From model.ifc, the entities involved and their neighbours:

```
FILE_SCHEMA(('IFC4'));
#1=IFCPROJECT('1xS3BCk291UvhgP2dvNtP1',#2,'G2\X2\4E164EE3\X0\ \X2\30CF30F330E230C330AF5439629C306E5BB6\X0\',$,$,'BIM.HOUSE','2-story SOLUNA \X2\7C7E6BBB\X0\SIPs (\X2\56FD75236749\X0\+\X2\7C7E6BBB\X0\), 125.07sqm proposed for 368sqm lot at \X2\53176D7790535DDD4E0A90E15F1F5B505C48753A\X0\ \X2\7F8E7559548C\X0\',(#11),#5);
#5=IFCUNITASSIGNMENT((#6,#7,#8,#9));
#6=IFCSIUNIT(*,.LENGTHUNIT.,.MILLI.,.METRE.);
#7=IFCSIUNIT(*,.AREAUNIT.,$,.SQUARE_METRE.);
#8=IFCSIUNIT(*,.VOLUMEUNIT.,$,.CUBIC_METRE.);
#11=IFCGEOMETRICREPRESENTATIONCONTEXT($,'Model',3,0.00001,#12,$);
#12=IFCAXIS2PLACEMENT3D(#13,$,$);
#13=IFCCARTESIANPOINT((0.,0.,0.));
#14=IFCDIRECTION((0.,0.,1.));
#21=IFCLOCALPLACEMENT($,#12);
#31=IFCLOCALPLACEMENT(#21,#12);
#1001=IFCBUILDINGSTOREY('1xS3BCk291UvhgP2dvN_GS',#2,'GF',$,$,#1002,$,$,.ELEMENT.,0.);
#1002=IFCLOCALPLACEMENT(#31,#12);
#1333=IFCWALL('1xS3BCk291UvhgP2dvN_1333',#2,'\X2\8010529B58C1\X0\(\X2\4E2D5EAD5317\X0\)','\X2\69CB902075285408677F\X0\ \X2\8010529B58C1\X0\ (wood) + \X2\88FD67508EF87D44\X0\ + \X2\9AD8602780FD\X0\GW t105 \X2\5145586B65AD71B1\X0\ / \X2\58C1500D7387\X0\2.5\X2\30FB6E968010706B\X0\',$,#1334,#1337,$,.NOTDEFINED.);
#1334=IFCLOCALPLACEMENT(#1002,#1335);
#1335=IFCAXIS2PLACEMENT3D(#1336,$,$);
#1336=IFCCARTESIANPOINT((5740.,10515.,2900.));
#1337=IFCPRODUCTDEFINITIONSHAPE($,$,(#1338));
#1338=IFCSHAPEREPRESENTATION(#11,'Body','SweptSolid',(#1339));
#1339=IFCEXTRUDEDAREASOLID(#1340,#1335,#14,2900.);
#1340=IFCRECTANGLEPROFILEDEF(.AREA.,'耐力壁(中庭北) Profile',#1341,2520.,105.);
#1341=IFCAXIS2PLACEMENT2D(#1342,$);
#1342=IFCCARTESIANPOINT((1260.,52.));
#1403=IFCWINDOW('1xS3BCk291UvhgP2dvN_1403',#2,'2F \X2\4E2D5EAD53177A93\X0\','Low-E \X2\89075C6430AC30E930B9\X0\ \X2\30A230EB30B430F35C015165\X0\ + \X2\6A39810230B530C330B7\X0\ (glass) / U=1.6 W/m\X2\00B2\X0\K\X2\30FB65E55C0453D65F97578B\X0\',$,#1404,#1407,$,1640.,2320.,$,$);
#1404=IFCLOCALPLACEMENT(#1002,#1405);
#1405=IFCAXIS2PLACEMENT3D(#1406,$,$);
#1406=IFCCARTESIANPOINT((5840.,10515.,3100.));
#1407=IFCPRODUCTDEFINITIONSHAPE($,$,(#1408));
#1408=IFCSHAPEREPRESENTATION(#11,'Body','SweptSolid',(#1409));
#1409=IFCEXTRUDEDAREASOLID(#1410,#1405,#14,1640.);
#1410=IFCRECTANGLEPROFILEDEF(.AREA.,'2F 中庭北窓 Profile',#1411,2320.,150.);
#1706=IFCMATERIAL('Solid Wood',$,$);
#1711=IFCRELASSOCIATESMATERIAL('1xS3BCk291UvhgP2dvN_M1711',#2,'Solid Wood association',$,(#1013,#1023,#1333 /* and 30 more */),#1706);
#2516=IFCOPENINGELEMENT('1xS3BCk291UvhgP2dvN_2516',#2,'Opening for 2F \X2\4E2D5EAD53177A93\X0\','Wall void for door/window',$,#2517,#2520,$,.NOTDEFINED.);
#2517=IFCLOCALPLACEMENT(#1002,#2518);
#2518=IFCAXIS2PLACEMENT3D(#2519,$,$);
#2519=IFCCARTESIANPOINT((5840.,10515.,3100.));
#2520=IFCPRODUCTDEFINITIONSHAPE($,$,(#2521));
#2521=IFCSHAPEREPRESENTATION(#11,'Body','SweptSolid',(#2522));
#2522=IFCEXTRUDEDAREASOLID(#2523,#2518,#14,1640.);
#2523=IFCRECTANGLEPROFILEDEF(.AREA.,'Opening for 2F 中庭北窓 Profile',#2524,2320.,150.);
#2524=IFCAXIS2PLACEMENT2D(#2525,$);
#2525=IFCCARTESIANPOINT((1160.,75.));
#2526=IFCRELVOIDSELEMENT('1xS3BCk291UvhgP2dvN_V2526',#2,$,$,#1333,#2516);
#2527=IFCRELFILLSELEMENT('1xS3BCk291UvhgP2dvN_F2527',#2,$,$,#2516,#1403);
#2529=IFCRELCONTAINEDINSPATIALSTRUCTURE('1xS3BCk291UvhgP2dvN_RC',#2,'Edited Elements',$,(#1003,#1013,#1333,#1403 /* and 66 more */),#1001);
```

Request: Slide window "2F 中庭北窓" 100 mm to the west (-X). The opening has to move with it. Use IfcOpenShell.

```python
import ifcopenshell
import ifcopenshell.api.geometry
import ifcopenshell.util.placement
import ifcopenshell.util.unit

model = ifcopenshell.open("model.ifc")
unit_scale = ifcopenshell.util.unit.calculate_unit_scale(model)

window = model.by_id(1403)
opening = window.FillsVoids[0].RelatingOpeningElement
wall = opening.VoidsElements[0].RelatingBuildingElement

wall_matrix = ifcopenshell.util.placement.get_local_placement(wall.ObjectPlacement)
shift = wall_matrix[:3, 0] * -0.1 / unit_scale
before = ifcopenshell.util.placement.get_local_placement(window.ObjectPlacement)[:3, 3].copy()

# The window is not placed relative to its opening, so move both.
for product in (opening, window):
    matrix = ifcopenshell.util.placement.get_local_placement(product.ObjectPlacement)
    matrix[:3, 3] += shift
    ifcopenshell.api.geometry.edit_object_placement(model, product=product, matrix=matrix, is_si=False)

after = ifcopenshell.util.placement.get_local_placement(window.ObjectPlacement)[:3, 3]
print("window moved by", (after - before).round(3) + 0.0)

model.write("model_edited.ifc")
```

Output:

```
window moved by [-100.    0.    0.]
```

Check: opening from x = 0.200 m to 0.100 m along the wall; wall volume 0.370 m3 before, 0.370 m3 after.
